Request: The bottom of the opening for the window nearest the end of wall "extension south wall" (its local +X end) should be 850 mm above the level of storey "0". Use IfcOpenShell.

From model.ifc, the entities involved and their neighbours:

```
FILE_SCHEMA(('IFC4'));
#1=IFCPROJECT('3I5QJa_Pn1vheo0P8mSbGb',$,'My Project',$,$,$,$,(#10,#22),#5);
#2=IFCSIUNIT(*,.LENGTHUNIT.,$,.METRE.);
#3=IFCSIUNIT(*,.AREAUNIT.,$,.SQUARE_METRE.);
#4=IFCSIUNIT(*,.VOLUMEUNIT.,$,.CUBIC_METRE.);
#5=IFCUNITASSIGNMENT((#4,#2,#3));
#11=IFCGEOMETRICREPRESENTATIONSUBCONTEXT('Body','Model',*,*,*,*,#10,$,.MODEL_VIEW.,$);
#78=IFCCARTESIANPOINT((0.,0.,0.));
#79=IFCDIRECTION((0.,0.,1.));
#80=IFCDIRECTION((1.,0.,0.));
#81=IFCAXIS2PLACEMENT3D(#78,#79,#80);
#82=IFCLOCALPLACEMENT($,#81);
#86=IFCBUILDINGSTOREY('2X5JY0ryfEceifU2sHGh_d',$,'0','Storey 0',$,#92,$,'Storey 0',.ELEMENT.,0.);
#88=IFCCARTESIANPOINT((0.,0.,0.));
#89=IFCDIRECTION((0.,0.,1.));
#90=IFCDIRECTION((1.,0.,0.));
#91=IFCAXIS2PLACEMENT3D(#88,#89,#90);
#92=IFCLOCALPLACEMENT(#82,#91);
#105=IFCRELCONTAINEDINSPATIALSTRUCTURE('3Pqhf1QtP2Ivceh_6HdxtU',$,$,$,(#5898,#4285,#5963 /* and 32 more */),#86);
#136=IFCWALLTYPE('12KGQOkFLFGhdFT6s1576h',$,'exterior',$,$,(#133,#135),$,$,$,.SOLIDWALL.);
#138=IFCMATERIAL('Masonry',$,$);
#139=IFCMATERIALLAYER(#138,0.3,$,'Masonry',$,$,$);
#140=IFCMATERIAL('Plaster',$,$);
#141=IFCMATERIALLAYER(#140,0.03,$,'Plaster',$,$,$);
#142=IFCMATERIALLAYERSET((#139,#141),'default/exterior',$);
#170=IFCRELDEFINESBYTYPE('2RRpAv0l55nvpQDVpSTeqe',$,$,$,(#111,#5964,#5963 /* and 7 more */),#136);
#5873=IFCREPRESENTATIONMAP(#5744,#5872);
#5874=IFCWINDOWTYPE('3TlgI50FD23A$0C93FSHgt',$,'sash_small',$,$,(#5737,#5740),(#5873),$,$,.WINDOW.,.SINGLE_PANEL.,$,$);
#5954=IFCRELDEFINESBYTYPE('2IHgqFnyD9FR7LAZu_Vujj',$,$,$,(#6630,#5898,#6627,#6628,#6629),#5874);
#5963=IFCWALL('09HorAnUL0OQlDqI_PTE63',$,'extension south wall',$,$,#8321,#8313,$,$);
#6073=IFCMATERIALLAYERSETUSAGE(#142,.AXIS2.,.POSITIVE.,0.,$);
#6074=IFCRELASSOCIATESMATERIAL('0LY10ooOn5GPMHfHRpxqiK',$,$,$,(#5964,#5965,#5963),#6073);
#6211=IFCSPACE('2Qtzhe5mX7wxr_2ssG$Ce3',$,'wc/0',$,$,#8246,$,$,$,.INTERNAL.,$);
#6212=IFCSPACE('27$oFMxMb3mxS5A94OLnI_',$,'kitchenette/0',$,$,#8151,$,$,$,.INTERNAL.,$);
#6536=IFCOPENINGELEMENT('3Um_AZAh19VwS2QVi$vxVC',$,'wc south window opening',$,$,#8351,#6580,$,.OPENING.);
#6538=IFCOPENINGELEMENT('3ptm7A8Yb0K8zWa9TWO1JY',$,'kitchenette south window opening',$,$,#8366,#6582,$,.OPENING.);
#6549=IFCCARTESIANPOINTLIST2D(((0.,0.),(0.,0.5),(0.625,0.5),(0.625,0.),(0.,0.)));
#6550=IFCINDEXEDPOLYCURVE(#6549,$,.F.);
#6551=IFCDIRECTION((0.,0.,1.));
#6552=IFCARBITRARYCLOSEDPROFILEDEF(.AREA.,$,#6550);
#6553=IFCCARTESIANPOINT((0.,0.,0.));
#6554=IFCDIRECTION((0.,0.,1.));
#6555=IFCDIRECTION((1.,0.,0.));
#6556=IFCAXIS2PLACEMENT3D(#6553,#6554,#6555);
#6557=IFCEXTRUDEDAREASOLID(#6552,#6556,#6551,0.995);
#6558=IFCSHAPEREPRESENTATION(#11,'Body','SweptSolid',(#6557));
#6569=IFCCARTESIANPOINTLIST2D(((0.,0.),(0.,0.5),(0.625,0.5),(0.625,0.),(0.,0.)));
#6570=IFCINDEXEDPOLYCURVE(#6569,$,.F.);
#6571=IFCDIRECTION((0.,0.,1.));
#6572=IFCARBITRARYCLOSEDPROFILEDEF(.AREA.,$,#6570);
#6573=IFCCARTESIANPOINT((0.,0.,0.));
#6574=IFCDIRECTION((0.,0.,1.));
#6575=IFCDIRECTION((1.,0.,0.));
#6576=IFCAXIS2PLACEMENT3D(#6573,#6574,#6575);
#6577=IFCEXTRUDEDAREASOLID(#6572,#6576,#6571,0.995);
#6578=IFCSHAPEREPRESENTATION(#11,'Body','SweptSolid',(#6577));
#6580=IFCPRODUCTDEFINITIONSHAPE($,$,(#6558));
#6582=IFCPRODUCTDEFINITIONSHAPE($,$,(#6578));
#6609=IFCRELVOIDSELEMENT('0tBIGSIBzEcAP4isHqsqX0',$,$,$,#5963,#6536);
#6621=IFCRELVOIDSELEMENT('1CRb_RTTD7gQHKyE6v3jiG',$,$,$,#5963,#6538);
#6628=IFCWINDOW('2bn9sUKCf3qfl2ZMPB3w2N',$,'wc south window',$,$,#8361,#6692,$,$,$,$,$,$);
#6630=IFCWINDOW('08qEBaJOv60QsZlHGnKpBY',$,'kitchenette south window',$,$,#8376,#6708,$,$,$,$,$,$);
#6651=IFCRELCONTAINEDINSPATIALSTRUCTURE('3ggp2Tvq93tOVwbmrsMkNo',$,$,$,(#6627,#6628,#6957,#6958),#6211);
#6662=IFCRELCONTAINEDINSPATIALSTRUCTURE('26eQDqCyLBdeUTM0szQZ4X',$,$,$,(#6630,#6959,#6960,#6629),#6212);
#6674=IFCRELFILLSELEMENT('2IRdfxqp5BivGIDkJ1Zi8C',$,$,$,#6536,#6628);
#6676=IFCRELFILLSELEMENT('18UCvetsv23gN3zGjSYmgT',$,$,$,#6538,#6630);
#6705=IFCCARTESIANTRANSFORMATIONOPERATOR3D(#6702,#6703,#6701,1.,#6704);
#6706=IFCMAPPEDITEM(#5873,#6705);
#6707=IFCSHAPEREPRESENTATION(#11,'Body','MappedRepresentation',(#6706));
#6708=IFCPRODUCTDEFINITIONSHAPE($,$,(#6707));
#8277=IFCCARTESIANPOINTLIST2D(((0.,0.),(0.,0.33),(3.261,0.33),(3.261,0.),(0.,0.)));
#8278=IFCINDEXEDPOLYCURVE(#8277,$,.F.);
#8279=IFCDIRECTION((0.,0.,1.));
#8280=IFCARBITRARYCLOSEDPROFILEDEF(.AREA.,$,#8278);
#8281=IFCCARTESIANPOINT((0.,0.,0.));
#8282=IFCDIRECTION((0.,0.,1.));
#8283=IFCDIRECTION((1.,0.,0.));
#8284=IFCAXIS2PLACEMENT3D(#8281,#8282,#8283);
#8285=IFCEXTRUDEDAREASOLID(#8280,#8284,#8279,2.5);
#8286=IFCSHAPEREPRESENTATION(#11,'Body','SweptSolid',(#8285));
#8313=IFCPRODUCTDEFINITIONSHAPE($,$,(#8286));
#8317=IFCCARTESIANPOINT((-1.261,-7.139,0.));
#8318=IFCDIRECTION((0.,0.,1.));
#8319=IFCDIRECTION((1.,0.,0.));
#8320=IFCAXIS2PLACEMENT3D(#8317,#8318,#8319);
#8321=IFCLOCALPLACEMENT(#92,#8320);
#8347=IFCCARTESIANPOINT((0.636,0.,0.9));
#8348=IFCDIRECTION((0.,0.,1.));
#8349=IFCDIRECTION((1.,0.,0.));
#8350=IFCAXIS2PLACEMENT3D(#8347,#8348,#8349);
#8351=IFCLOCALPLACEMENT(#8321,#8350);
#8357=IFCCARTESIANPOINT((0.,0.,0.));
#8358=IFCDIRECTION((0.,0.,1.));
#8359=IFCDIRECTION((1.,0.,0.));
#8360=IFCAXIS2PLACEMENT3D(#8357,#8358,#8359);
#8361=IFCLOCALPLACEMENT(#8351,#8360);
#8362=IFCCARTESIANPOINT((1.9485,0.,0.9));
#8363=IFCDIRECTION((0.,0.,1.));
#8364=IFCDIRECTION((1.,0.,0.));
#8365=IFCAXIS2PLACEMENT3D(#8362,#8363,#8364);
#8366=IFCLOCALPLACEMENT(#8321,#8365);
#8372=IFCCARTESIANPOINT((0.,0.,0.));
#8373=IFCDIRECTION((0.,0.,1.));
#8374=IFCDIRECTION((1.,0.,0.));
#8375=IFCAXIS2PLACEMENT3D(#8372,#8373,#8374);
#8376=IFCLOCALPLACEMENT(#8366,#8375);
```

```python
import numpy as np
import ifcopenshell
import ifcopenshell.api.geometry
import ifcopenshell.geom
import ifcopenshell.util.element
import ifcopenshell.util.placement
import ifcopenshell.util.shape
import ifcopenshell.util.unit

model = ifcopenshell.open("model.ifc")
unit_scale = ifcopenshell.util.unit.calculate_unit_scale(model)

window = model.by_id(6630)
opening = window.FillsVoids[0].RelatingOpeningElement
storey = ifcopenshell.util.element.get_container(window, ifc_class="IfcBuildingStorey")
level = ifcopenshell.util.placement.get_local_placement(storey.ObjectPlacement)[2, 3]

# The opening's origin need not be at the sill, so measure its lowest point.
shape = ifcopenshell.geom.create_shape(ifcopenshell.geom.settings(), opening)
bottom = ifcopenshell.util.shape.get_shape_bottom_elevation(shape, shape.geometry) / unit_scale
dz = level + 0.85 - bottom

shift = np.array([0.0, 0.0, dz])
# The window is placed relative to its opening, so it follows when the opening moves.
matrix = ifcopenshell.util.placement.get_local_placement(opening.ObjectPlacement)
matrix[:3, 3] += shift
ifcopenshell.api.geometry.edit_object_placement(
    model, product=opening, matrix=matrix, is_si=False, should_transform_children=True
)

print(f"moved by {dz * unit_scale:+.3f} m")

model.write("model_rev.ifc")
```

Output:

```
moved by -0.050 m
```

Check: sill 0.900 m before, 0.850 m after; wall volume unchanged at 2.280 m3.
